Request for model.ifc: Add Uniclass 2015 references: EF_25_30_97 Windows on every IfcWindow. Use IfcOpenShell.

First a look at what the model holds.

```python
import ifcopenshell

model = ifcopenshell.open("model.ifc")
print(model.schema)
print("classifications:", [c.Name for c in model.by_type("IfcClassification")])
for ifc_class in ("IfcDoor", "IfcRoof", "IfcStair", "IfcWall", "IfcWindow"):
    print(ifc_class, len(model.by_type(ifc_class)))
```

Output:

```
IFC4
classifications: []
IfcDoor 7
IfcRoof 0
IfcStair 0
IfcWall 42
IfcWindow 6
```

```python
import ifcopenshell
import ifcopenshell.api.classification

model = ifcopenshell.open("model.ifc")

system = ifcopenshell.api.classification.add_classification(model, classification="Uniclass 2015")

codes = {
    "IfcWindow": ("EF_25_30_97", "Windows"),
}
for ifc_class, (code, name) in codes.items():
    products = model.by_type(ifc_class)
    ifcopenshell.api.classification.add_reference(
        model, products=products, classification=system, identification=code, name=name
    )
    print(code, len(products))

model.write("model_edited.ifc")
```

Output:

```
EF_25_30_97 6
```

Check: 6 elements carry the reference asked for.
